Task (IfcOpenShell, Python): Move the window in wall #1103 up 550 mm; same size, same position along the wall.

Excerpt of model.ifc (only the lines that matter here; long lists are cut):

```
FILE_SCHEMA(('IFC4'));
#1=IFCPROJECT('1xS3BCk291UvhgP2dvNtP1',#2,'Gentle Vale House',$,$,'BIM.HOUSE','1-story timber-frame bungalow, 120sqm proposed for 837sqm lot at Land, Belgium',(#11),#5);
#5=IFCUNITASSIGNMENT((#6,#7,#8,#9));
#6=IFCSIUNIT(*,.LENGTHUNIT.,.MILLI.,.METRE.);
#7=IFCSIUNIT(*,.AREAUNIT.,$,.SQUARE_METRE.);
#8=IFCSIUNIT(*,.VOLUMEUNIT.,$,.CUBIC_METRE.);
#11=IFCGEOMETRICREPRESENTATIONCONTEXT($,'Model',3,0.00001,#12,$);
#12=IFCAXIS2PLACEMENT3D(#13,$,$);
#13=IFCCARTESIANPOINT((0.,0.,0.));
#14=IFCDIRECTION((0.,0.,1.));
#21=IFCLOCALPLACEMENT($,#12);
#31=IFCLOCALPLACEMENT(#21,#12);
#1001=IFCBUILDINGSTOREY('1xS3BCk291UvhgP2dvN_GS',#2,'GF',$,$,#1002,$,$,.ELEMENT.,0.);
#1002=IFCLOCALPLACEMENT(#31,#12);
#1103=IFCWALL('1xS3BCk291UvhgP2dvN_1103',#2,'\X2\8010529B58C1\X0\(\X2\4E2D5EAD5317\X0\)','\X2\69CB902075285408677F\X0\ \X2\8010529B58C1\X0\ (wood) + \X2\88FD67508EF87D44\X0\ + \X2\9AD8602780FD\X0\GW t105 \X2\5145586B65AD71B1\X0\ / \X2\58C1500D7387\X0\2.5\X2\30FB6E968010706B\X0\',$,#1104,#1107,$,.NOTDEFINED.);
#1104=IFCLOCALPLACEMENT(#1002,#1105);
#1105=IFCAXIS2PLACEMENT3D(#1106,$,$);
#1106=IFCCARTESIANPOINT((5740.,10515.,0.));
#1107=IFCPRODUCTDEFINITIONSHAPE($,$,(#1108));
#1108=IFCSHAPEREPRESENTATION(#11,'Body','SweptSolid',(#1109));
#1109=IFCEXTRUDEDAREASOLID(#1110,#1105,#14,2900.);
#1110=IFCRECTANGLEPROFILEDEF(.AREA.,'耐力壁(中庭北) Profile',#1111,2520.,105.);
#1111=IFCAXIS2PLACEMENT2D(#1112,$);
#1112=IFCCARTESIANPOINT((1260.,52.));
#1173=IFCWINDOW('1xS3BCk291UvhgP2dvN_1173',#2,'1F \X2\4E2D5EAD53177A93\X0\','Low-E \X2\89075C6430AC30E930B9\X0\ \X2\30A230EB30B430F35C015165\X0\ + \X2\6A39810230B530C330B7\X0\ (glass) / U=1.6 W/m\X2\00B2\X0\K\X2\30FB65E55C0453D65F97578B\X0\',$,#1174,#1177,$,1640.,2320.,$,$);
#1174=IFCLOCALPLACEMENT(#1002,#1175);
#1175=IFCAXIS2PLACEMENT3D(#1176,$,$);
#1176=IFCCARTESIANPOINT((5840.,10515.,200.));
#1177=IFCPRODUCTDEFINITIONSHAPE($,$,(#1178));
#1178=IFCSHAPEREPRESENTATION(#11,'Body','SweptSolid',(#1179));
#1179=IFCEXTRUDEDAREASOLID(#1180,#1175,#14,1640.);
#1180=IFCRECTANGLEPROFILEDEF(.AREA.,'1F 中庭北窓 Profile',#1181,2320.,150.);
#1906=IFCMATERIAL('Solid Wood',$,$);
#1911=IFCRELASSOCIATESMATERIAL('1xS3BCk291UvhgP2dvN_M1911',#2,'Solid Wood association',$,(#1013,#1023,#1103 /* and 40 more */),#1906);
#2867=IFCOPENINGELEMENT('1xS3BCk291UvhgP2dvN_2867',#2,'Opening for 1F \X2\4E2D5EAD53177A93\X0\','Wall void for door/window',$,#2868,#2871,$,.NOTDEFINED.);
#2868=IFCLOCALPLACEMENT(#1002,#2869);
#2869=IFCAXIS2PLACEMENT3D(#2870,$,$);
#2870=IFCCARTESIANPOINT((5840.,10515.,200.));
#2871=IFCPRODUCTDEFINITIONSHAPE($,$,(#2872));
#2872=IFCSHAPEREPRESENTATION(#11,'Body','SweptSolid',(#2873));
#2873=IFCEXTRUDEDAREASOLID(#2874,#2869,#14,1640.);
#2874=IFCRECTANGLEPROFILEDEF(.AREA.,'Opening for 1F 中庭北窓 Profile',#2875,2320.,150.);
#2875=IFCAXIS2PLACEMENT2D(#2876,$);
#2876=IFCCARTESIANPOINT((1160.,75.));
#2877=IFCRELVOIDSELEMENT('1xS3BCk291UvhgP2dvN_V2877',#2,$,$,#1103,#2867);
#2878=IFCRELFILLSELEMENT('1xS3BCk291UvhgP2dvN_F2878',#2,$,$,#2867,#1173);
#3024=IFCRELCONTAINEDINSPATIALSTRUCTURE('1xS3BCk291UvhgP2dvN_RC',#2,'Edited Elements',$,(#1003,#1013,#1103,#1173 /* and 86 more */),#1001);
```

```python
import numpy as np
import ifcopenshell
import ifcopenshell.api.geometry
import ifcopenshell.util.placement
import ifcopenshell.util.unit

model = ifcopenshell.open("model.ifc")
unit_scale = ifcopenshell.util.unit.calculate_unit_scale(model)

window = model.by_guid("1xS3BCk291UvhgP2dvN_1173")
opening = window.FillsVoids[0].RelatingOpeningElement
dz = 550.0

shift = np.array([0.0, 0.0, dz])
# The window is not placed relative to its opening, so move both.
for product in (opening, window):
    matrix = ifcopenshell.util.placement.get_local_placement(product.ObjectPlacement)
    matrix[:3, 3] += shift
    ifcopenshell.api.geometry.edit_object_placement(model, product=product, matrix=matrix, is_si=False)

print(f"moved by {dz * unit_scale:+.3f} m")

model.write("model_v2.ifc")
```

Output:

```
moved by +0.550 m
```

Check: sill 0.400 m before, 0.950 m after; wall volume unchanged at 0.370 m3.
